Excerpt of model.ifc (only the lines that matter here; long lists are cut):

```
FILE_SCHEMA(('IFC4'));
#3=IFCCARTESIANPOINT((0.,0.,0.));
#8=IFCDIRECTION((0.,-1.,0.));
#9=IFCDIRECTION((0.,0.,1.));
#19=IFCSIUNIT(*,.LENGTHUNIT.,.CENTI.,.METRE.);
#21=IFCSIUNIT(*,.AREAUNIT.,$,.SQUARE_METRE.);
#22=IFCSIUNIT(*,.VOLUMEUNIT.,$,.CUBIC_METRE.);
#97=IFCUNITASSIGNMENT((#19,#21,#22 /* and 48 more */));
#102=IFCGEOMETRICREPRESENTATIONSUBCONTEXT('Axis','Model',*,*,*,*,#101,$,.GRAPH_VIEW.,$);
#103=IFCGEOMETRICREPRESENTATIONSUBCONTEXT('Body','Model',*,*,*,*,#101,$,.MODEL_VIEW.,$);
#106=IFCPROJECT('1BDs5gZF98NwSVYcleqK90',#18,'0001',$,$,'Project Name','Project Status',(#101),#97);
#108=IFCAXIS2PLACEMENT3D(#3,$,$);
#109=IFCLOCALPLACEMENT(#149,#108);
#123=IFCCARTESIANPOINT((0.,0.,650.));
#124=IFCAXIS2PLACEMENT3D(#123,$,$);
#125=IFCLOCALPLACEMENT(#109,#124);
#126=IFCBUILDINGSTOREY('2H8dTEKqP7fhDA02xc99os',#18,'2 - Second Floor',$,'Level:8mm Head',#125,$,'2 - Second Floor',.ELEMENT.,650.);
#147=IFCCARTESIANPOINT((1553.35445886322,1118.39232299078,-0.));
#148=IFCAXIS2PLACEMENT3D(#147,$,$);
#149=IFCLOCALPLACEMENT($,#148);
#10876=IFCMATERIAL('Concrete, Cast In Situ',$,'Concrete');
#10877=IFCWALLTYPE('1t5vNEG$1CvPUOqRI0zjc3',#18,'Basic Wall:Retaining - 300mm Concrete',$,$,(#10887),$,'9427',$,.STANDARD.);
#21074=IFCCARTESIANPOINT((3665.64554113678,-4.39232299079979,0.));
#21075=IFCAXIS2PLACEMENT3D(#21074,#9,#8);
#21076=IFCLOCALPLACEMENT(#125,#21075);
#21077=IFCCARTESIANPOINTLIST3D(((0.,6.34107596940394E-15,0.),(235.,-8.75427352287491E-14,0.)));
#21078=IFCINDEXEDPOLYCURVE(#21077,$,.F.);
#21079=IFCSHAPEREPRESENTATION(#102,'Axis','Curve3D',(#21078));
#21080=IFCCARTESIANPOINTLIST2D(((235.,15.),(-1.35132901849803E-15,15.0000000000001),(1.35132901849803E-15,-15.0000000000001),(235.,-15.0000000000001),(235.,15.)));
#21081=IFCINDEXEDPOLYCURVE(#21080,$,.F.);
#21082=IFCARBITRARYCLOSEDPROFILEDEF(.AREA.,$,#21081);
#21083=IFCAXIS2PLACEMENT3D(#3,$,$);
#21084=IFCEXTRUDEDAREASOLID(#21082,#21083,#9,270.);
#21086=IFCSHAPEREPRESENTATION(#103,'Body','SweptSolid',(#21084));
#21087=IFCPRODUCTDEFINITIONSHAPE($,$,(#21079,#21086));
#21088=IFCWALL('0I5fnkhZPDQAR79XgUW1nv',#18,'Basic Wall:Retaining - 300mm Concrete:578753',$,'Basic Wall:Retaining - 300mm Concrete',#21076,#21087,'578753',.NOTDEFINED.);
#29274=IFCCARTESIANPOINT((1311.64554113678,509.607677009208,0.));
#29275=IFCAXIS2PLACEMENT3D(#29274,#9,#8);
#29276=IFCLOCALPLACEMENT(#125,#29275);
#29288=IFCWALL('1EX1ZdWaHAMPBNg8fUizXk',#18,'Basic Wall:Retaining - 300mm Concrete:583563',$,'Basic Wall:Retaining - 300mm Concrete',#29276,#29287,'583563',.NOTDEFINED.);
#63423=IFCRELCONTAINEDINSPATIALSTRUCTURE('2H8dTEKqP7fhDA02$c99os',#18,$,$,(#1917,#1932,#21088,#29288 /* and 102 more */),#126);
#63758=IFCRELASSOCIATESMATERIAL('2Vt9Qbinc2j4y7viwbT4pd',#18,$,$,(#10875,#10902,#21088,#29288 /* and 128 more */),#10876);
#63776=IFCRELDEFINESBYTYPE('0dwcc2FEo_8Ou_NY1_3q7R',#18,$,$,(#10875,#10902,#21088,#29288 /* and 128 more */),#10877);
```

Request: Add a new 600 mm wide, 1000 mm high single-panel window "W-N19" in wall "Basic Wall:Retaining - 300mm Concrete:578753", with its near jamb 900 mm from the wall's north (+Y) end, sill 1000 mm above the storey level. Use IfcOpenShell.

```python
import numpy as np
import ifcopenshell
import ifcopenshell.api.feature
import ifcopenshell.api.geometry
import ifcopenshell.api.root
import ifcopenshell.api.spatial
import ifcopenshell.geom
import ifcopenshell.util.element
import ifcopenshell.util.placement
import ifcopenshell.util.representation
import ifcopenshell.util.shape
import ifcopenshell.util.unit

model = ifcopenshell.open("model.ifc")
unit_scale = ifcopenshell.util.unit.calculate_unit_scale(model)
settings = ifcopenshell.geom.settings()


def volume(element):
    """Net volume in cubic metres, openings subtracted."""
    shape = ifcopenshell.geom.create_shape(settings, element)
    return ifcopenshell.util.shape.get_volume(shape.geometry)


wall = model.by_id(21088)
storey = ifcopenshell.util.element.get_container(wall, ifc_class="IfcBuildingStorey")
context = ifcopenshell.util.representation.get_context(model, "Model", "Body", "MODEL_VIEW")
before = volume(wall)

width, height, from_end, sill = 0.6, 1, 0.9, 1  # metres

# The wall runs along its own X axis, and the end named is its -X end.
wall_shape = ifcopenshell.geom.create_shape(settings, wall)
x, y, z = ifcopenshell.util.shape.get_vertices(wall_shape.geometry).T
start = x.min() + from_end
face, thickness = float(y.min()), float(y.max() - y.min())
wall_matrix = ifcopenshell.util.placement.get_local_placement(wall.ObjectPlacement)
level = ifcopenshell.util.placement.get_local_placement(storey.ObjectPlacement)[2, 3]


def in_wall(x, y):
    """Placement at x, y metres in the wall's axes, at sill height."""
    matrix = wall_matrix.copy()
    matrix[:, 3] = wall_matrix @ np.array([x / unit_scale, y / unit_scale, 0.0, 1.0])
    matrix[2, 3] = level + sill / unit_scale
    return matrix


# Opening: a box that overshoots both wall faces by 50 mm.
opening = ifcopenshell.api.root.create_entity(model, ifc_class="IfcOpeningElement", predefined_type="OPENING")
box = ifcopenshell.api.geometry.add_wall_representation(
    model, context=context, length=width, height=height, thickness=thickness + 0.1
)
ifcopenshell.api.geometry.assign_representation(model, product=opening, representation=box)
ifcopenshell.api.geometry.edit_object_placement(model, product=opening, matrix=in_wall(start, face - 0.05), is_si=False)
ifcopenshell.api.feature.add_feature(model, feature=opening, element=wall)

window = ifcopenshell.api.root.create_entity(model, ifc_class="IfcWindow", name="W-N19", predefined_type="WINDOW")
window.OverallWidth, window.OverallHeight = width / unit_scale, height / unit_scale
window.PartitioningType = "SINGLE_PANEL"
body = ifcopenshell.api.geometry.add_window_representation(
    model,
    context=context,
    overall_width=window.OverallWidth,
    overall_height=window.OverallHeight,
    partition_type="SINGLE_PANEL",
)
ifcopenshell.api.geometry.assign_representation(model, product=window, representation=body)
ifcopenshell.api.spatial.assign_container(model, products=[window], relating_structure=storey)
ifcopenshell.api.feature.add_filling(model, opening=opening, element=window)

# Centre the window in the wall's thickness.
ifcopenshell.api.geometry.edit_object_placement(model, product=window, matrix=in_wall(start, face), is_si=False)
window_shape = ifcopenshell.geom.create_shape(settings, window)
depth = ifcopenshell.util.shape.get_vertices(window_shape.geometry)[:, 1]
offset = face + thickness / 2 - (depth.min() + depth.max()) / 2
ifcopenshell.api.geometry.edit_object_placement(model, product=window, matrix=in_wall(start, offset), is_si=False)

after = volume(wall)

print(f"wall volume {before:.3f} -> {after:.3f} m3")

model.write("model-out.ifc")
```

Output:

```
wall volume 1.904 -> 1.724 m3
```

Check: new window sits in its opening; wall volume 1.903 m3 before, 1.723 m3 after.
